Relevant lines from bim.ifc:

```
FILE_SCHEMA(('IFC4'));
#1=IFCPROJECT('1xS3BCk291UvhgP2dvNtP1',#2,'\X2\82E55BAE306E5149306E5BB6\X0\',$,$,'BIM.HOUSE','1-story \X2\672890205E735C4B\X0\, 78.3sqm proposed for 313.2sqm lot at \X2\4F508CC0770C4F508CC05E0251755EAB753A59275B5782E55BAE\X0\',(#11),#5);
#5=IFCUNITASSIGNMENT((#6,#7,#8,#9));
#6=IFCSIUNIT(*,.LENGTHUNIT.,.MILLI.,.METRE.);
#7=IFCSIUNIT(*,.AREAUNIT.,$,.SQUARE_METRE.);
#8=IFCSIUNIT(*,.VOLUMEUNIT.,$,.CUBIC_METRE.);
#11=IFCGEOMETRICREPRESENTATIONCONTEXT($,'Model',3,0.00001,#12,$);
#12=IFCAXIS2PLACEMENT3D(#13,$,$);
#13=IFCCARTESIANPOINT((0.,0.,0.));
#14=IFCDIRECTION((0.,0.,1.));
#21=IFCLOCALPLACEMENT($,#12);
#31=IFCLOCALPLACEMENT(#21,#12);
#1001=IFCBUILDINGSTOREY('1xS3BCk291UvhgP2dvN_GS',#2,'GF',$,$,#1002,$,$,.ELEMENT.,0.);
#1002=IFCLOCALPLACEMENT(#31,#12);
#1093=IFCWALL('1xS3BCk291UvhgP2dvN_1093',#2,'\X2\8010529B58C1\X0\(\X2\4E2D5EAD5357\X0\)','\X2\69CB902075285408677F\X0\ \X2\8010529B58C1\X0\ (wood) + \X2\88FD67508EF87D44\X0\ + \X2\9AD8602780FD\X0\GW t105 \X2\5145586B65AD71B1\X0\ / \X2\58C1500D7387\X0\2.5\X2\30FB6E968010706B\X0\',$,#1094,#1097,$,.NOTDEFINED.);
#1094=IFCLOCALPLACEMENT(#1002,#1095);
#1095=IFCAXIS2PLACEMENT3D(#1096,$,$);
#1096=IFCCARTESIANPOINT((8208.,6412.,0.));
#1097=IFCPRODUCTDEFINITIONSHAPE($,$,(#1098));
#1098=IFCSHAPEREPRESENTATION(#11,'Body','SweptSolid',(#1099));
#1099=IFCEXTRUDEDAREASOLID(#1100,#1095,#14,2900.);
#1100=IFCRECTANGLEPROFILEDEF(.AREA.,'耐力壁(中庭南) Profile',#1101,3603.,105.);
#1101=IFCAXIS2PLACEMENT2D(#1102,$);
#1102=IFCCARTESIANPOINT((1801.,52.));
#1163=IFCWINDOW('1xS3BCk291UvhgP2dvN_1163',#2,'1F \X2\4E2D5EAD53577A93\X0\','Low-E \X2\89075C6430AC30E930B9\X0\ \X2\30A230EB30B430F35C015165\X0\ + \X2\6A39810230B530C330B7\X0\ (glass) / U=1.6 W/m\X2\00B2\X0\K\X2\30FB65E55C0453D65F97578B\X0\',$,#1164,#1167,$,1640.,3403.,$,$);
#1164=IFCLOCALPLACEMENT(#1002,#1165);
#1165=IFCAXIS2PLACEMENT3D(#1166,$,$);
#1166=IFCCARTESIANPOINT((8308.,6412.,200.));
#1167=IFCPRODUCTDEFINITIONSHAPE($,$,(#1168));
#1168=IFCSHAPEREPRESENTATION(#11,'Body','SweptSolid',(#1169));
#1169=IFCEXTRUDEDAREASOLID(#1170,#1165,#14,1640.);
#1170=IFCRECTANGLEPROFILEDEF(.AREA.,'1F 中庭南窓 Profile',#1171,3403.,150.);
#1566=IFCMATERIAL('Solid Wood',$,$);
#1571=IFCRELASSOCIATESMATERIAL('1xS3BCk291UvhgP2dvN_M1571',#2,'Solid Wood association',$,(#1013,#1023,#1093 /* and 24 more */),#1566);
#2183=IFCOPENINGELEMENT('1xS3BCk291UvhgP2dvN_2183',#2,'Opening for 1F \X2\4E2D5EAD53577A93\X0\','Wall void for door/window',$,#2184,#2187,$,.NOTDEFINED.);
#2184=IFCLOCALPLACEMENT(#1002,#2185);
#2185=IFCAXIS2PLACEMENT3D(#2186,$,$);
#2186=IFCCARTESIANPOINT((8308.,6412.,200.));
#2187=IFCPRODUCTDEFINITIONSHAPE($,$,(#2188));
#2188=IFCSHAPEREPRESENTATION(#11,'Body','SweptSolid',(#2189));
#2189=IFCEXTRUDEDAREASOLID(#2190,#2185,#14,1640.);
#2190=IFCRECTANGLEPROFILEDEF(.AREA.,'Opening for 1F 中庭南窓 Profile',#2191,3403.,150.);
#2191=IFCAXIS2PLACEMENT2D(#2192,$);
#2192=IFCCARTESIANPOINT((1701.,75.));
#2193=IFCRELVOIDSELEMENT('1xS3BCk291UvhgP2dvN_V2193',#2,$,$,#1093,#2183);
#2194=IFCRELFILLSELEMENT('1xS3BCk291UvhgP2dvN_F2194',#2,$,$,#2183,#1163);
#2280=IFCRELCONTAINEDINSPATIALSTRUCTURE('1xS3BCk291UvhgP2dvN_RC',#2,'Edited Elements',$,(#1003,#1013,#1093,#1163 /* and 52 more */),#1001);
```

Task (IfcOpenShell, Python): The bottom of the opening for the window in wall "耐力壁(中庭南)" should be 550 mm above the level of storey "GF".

```python
import numpy as np
import ifcopenshell
import ifcopenshell.api.geometry
import ifcopenshell.geom
import ifcopenshell.util.element
import ifcopenshell.util.placement
import ifcopenshell.util.shape
import ifcopenshell.util.unit

model = ifcopenshell.open("bim.ifc")
unit_scale = ifcopenshell.util.unit.calculate_unit_scale(model)

window = model.by_guid("1xS3BCk291UvhgP2dvN_1163")
opening = window.FillsVoids[0].RelatingOpeningElement
storey = ifcopenshell.util.element.get_container(window, ifc_class="IfcBuildingStorey")
level = ifcopenshell.util.placement.get_local_placement(storey.ObjectPlacement)[2, 3]

# The opening's origin need not be at the sill, so measure its lowest point.
shape = ifcopenshell.geom.create_shape(ifcopenshell.geom.settings(), opening)
bottom = ifcopenshell.util.shape.get_shape_bottom_elevation(shape, shape.geometry) / unit_scale
dz = level + 0.55 / unit_scale - bottom

shift = np.array([0.0, 0.0, dz])
# The window is not placed relative to its opening, so move both.
for product in (opening, window):
    matrix = ifcopenshell.util.placement.get_local_placement(product.ObjectPlacement)
    matrix[:3, 3] += shift
    ifcopenshell.api.geometry.edit_object_placement(model, product=product, matrix=matrix, is_si=False)

print(f"moved by {dz * unit_scale:+.3f} m")

model.write("bim_updated.ifc")
```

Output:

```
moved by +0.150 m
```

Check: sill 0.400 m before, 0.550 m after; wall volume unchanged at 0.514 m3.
